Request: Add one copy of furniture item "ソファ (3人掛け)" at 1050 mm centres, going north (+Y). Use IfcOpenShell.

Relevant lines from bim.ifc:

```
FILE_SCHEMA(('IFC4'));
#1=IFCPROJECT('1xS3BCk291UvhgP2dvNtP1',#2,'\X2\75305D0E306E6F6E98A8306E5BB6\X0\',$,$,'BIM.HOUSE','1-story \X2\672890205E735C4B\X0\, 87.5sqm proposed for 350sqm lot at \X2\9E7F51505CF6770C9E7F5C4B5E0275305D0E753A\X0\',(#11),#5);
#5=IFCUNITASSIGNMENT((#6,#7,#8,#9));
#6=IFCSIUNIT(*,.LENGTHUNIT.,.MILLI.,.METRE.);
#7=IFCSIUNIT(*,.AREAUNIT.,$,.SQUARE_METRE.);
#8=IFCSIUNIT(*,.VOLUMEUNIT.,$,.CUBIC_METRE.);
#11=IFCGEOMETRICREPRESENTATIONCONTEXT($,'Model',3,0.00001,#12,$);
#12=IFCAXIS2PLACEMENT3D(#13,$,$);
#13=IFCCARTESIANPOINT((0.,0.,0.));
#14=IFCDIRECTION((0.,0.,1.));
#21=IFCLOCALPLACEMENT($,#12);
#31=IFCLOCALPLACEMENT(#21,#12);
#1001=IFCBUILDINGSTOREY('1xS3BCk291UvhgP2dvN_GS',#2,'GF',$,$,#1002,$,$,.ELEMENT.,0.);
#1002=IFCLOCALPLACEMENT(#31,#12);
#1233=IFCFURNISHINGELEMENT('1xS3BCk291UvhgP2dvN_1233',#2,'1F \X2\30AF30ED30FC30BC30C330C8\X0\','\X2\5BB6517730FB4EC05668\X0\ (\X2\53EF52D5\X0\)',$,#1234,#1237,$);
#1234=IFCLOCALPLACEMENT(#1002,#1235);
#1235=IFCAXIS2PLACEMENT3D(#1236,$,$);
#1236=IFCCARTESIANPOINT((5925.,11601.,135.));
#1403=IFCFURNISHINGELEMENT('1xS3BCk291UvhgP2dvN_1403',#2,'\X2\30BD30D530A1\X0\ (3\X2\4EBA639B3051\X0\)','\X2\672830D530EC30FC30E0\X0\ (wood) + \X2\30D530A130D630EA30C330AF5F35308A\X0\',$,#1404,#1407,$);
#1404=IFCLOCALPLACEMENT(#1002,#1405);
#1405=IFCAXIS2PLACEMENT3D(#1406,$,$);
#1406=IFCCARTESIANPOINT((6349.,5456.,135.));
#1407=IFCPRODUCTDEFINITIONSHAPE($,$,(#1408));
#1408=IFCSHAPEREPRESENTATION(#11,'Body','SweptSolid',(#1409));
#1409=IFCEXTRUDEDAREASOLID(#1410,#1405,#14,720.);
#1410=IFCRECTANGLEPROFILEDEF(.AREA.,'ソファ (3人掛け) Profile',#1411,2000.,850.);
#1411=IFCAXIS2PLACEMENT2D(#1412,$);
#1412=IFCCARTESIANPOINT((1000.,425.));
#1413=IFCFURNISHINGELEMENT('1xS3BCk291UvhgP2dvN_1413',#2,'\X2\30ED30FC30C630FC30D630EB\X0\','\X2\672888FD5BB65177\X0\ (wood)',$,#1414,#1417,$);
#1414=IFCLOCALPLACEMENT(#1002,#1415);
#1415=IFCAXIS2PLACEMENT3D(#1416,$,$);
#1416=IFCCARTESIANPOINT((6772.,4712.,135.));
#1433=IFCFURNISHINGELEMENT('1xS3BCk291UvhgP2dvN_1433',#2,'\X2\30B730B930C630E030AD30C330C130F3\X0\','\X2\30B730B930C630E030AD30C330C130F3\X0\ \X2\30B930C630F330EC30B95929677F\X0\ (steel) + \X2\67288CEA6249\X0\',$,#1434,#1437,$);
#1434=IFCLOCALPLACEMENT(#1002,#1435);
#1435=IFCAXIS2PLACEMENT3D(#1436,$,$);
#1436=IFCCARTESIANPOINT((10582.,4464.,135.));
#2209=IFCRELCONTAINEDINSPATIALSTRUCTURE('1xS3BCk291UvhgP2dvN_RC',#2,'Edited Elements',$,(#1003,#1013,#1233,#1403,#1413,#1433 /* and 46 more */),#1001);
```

```python
import numpy as np
import ifcopenshell
import ifcopenshell.api.geometry
import ifcopenshell.api.root
import ifcopenshell.util.element
import ifcopenshell.util.placement

model = ifcopenshell.open("bim.ifc")


def reuse_history(source, copy):
    """copy_class also copies each property set's owner history, people and application; keep the originals."""
    for rel in copy.IsDefinedBy:
        if rel.is_a("IfcRelDefinesByProperties") and (history := rel.RelatingPropertyDefinition.OwnerHistory):
            rel.RelatingPropertyDefinition.OwnerHistory = source.OwnerHistory
            ifcopenshell.util.element.remove_deep2(model, history)


source = model.by_guid("1xS3BCk291UvhgP2dvN_1403")
base = ifcopenshell.util.placement.get_local_placement(source.ObjectPlacement)
step = np.array([0.0, 1.0, 0.0]) * 1050.0

for i in range(1, 2):
    copy = ifcopenshell.api.root.copy_class(model, product=source)
    copy.Representation = ifcopenshell.util.element.copy_deep(
        model, source.Representation, exclude=["IfcGeometricRepresentationContext", "IfcRepresentationMap"]
    )
    reuse_history(source, copy)
    matrix = base.copy()
    matrix[:3, 3] += i * step
    print("added at", matrix[:3, 3].round(3) + 0.0)
    ifcopenshell.api.geometry.edit_object_placement(model, product=copy, matrix=matrix, is_si=False)

model.write("bim-out.ifc")
```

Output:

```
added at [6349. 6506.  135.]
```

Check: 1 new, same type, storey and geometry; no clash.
